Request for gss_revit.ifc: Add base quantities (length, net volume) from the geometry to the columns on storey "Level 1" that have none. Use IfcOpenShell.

First a look at what the model holds.

```python
import ifcopenshell
import ifcopenshell.util.element
import ifcopenshell.util.unit

model = ifcopenshell.open("gss_revit.ifc")
print(model.schema)
for unit_type in ("LENGTHUNIT", "AREAUNIT", "VOLUMEUNIT"):
    print(unit_type, ifcopenshell.util.unit.calculate_unit_scale(model, unit_type))
storey = next(s for s in model.by_type("IfcBuildingStorey") if s.Name == "Level 1")
columns = [e for e in ifcopenshell.util.element.get_decomposition(storey) if e.is_a("IfcColumn")]
for e in sorted(columns, key=lambda e: e.id()):
    print(e.id(), e.is_a(), e.Name, list(ifcopenshell.util.element.get_psets(e, qtos_only=True)), sep=" | ")
```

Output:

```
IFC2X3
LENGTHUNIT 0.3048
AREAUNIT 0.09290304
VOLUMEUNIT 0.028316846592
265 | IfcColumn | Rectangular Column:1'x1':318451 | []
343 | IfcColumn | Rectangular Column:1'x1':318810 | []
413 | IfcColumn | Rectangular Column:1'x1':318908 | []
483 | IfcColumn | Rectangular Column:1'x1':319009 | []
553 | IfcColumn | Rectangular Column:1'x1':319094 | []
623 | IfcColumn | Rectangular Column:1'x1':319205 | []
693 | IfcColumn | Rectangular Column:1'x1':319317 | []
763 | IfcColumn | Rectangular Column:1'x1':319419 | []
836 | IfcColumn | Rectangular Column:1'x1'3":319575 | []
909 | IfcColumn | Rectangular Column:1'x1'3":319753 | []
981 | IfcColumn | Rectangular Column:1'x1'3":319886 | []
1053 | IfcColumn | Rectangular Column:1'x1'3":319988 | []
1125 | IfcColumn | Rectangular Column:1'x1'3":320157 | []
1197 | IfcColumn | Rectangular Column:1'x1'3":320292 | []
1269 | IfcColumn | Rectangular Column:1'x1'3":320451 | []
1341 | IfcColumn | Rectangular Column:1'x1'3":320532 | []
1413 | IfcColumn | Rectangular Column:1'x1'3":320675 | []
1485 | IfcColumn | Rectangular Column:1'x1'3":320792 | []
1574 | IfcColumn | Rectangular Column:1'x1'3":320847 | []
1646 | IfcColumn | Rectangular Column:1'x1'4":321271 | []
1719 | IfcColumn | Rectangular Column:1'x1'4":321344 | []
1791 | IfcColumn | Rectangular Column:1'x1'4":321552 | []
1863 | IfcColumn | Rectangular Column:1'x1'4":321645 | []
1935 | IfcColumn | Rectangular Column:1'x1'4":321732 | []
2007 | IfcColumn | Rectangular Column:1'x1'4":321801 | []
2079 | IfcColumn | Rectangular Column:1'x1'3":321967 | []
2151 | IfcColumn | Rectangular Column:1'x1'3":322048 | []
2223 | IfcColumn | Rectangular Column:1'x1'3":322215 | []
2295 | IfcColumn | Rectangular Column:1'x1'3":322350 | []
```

```python
import ifcopenshell
import ifcopenshell.api.pset
import ifcopenshell.geom
import ifcopenshell.util.element
import ifcopenshell.util.shape
import ifcopenshell.util.unit

model = ifcopenshell.open("gss_revit.ifc")
unit_scale = ifcopenshell.util.unit.calculate_unit_scale(model)
volume_scale = ifcopenshell.util.unit.calculate_unit_scale(model, "VOLUMEUNIT")
settings = ifcopenshell.geom.settings()

storey = next(s for s in model.by_type("IfcBuildingStorey") if s.Name == "Level 1")
columns = [e for e in ifcopenshell.util.element.get_decomposition(storey) if e.is_a("IfcColumn")]

for e in sorted(columns, key=lambda e: e.id()):
    if ifcopenshell.util.element.get_psets(e, qtos_only=True, should_inherit=False):
        continue
    # Geometry comes back in metres, in the element's own axes.
    shape = ifcopenshell.geom.create_shape(settings, e)
    values = {
        "Length": ifcopenshell.util.shape.get_z(shape.geometry) / unit_scale,
        "NetVolume": ifcopenshell.util.shape.get_volume(shape.geometry) / volume_scale,
    }
    qto = ifcopenshell.api.pset.add_qto(model, product=e, name="BaseQuantities")
    ifcopenshell.api.pset.edit_qto(model, qto=qto, properties=values)
    print(e.id(), {k: round(v, 3) for k, v in values.items()})

model.write("gss_revit_updated.ifc")
```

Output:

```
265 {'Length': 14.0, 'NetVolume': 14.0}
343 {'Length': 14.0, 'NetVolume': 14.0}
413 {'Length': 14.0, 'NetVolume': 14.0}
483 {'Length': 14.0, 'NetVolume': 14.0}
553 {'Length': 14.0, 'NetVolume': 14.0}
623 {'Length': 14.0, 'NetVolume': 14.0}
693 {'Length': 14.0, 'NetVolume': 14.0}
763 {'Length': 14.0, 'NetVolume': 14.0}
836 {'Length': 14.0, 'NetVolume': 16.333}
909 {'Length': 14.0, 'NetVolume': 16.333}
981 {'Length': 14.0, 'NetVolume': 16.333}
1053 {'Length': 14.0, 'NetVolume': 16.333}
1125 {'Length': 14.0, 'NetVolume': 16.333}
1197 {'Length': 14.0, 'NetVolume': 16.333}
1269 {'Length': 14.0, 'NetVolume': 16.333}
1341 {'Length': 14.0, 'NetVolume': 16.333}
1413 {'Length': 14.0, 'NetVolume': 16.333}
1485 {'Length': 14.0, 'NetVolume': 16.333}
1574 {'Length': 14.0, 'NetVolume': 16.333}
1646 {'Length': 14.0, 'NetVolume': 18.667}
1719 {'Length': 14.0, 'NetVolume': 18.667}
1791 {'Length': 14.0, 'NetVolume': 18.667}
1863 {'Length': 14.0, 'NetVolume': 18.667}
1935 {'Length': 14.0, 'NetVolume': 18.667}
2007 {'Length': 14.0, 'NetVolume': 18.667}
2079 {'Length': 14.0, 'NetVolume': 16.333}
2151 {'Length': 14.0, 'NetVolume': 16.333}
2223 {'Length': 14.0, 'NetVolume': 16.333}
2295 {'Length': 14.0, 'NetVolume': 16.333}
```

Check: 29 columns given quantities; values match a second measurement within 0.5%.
